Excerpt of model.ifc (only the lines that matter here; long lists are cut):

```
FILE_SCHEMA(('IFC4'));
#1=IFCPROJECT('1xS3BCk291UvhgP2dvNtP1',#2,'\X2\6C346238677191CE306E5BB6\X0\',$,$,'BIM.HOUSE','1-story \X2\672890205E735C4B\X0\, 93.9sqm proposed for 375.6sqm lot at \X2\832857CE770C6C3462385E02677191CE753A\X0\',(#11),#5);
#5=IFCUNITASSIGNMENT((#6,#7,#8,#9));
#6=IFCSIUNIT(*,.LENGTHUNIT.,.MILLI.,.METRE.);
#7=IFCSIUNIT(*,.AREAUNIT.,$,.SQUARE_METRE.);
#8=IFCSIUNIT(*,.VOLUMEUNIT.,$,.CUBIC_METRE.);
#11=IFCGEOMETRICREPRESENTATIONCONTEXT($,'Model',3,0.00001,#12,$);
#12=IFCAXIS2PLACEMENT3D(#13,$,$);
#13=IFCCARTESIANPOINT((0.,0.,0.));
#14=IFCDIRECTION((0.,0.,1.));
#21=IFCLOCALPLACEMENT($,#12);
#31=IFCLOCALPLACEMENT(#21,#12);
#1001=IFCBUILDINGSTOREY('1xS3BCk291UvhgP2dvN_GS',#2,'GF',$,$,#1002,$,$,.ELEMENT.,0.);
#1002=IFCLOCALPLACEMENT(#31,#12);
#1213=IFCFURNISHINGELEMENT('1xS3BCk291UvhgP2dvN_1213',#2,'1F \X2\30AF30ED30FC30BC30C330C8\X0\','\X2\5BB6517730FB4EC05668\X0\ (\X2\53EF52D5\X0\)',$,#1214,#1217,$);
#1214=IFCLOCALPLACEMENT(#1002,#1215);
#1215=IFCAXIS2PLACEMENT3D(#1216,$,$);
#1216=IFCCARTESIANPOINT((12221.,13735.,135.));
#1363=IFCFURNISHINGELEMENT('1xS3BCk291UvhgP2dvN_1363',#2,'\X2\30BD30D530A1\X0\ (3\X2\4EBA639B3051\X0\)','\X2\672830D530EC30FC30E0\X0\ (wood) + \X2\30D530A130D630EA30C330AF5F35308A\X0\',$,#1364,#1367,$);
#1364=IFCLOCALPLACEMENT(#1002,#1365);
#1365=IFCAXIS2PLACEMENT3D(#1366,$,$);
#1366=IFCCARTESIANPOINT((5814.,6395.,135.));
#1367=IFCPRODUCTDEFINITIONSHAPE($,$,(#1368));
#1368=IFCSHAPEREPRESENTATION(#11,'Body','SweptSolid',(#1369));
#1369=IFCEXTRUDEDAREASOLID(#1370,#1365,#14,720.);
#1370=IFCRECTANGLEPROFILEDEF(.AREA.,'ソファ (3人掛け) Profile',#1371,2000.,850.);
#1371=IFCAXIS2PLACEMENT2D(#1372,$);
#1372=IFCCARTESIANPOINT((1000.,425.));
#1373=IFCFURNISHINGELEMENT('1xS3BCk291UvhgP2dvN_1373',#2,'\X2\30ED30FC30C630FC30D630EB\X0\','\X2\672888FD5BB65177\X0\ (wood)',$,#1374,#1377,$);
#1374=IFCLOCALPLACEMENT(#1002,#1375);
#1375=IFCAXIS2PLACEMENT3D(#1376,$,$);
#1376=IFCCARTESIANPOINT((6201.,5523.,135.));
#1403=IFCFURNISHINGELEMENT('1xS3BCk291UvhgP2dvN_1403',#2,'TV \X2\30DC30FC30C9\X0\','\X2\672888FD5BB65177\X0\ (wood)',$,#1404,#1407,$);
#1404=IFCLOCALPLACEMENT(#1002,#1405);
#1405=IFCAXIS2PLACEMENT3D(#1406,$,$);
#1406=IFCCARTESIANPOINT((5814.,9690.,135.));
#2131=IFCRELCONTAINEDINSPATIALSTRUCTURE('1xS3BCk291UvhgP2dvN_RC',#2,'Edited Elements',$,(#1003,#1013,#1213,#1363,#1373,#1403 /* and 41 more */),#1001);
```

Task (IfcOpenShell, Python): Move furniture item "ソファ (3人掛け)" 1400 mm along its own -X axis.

```python
import ifcopenshell
import ifcopenshell.api.geometry
import ifcopenshell.util.placement
import ifcopenshell.util.unit

model = ifcopenshell.open("model.ifc")
unit_scale = ifcopenshell.util.unit.calculate_unit_scale(model)

item = model.by_id(1363)
matrix = ifcopenshell.util.placement.get_local_placement(item.ObjectPlacement)
matrix[:3, 3] -= matrix[:3, 0] * 1.4 / unit_scale
ifcopenshell.api.geometry.edit_object_placement(model, product=item, matrix=matrix, is_si=False)

print(ifcopenshell.util.placement.get_local_placement(item.ObjectPlacement).round(3) + 0.0)

model.write("model_updated.ifc")
```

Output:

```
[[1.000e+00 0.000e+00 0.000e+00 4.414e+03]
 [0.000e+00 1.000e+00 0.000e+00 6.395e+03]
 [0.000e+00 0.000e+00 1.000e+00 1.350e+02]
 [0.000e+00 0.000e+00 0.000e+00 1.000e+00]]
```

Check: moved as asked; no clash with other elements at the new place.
